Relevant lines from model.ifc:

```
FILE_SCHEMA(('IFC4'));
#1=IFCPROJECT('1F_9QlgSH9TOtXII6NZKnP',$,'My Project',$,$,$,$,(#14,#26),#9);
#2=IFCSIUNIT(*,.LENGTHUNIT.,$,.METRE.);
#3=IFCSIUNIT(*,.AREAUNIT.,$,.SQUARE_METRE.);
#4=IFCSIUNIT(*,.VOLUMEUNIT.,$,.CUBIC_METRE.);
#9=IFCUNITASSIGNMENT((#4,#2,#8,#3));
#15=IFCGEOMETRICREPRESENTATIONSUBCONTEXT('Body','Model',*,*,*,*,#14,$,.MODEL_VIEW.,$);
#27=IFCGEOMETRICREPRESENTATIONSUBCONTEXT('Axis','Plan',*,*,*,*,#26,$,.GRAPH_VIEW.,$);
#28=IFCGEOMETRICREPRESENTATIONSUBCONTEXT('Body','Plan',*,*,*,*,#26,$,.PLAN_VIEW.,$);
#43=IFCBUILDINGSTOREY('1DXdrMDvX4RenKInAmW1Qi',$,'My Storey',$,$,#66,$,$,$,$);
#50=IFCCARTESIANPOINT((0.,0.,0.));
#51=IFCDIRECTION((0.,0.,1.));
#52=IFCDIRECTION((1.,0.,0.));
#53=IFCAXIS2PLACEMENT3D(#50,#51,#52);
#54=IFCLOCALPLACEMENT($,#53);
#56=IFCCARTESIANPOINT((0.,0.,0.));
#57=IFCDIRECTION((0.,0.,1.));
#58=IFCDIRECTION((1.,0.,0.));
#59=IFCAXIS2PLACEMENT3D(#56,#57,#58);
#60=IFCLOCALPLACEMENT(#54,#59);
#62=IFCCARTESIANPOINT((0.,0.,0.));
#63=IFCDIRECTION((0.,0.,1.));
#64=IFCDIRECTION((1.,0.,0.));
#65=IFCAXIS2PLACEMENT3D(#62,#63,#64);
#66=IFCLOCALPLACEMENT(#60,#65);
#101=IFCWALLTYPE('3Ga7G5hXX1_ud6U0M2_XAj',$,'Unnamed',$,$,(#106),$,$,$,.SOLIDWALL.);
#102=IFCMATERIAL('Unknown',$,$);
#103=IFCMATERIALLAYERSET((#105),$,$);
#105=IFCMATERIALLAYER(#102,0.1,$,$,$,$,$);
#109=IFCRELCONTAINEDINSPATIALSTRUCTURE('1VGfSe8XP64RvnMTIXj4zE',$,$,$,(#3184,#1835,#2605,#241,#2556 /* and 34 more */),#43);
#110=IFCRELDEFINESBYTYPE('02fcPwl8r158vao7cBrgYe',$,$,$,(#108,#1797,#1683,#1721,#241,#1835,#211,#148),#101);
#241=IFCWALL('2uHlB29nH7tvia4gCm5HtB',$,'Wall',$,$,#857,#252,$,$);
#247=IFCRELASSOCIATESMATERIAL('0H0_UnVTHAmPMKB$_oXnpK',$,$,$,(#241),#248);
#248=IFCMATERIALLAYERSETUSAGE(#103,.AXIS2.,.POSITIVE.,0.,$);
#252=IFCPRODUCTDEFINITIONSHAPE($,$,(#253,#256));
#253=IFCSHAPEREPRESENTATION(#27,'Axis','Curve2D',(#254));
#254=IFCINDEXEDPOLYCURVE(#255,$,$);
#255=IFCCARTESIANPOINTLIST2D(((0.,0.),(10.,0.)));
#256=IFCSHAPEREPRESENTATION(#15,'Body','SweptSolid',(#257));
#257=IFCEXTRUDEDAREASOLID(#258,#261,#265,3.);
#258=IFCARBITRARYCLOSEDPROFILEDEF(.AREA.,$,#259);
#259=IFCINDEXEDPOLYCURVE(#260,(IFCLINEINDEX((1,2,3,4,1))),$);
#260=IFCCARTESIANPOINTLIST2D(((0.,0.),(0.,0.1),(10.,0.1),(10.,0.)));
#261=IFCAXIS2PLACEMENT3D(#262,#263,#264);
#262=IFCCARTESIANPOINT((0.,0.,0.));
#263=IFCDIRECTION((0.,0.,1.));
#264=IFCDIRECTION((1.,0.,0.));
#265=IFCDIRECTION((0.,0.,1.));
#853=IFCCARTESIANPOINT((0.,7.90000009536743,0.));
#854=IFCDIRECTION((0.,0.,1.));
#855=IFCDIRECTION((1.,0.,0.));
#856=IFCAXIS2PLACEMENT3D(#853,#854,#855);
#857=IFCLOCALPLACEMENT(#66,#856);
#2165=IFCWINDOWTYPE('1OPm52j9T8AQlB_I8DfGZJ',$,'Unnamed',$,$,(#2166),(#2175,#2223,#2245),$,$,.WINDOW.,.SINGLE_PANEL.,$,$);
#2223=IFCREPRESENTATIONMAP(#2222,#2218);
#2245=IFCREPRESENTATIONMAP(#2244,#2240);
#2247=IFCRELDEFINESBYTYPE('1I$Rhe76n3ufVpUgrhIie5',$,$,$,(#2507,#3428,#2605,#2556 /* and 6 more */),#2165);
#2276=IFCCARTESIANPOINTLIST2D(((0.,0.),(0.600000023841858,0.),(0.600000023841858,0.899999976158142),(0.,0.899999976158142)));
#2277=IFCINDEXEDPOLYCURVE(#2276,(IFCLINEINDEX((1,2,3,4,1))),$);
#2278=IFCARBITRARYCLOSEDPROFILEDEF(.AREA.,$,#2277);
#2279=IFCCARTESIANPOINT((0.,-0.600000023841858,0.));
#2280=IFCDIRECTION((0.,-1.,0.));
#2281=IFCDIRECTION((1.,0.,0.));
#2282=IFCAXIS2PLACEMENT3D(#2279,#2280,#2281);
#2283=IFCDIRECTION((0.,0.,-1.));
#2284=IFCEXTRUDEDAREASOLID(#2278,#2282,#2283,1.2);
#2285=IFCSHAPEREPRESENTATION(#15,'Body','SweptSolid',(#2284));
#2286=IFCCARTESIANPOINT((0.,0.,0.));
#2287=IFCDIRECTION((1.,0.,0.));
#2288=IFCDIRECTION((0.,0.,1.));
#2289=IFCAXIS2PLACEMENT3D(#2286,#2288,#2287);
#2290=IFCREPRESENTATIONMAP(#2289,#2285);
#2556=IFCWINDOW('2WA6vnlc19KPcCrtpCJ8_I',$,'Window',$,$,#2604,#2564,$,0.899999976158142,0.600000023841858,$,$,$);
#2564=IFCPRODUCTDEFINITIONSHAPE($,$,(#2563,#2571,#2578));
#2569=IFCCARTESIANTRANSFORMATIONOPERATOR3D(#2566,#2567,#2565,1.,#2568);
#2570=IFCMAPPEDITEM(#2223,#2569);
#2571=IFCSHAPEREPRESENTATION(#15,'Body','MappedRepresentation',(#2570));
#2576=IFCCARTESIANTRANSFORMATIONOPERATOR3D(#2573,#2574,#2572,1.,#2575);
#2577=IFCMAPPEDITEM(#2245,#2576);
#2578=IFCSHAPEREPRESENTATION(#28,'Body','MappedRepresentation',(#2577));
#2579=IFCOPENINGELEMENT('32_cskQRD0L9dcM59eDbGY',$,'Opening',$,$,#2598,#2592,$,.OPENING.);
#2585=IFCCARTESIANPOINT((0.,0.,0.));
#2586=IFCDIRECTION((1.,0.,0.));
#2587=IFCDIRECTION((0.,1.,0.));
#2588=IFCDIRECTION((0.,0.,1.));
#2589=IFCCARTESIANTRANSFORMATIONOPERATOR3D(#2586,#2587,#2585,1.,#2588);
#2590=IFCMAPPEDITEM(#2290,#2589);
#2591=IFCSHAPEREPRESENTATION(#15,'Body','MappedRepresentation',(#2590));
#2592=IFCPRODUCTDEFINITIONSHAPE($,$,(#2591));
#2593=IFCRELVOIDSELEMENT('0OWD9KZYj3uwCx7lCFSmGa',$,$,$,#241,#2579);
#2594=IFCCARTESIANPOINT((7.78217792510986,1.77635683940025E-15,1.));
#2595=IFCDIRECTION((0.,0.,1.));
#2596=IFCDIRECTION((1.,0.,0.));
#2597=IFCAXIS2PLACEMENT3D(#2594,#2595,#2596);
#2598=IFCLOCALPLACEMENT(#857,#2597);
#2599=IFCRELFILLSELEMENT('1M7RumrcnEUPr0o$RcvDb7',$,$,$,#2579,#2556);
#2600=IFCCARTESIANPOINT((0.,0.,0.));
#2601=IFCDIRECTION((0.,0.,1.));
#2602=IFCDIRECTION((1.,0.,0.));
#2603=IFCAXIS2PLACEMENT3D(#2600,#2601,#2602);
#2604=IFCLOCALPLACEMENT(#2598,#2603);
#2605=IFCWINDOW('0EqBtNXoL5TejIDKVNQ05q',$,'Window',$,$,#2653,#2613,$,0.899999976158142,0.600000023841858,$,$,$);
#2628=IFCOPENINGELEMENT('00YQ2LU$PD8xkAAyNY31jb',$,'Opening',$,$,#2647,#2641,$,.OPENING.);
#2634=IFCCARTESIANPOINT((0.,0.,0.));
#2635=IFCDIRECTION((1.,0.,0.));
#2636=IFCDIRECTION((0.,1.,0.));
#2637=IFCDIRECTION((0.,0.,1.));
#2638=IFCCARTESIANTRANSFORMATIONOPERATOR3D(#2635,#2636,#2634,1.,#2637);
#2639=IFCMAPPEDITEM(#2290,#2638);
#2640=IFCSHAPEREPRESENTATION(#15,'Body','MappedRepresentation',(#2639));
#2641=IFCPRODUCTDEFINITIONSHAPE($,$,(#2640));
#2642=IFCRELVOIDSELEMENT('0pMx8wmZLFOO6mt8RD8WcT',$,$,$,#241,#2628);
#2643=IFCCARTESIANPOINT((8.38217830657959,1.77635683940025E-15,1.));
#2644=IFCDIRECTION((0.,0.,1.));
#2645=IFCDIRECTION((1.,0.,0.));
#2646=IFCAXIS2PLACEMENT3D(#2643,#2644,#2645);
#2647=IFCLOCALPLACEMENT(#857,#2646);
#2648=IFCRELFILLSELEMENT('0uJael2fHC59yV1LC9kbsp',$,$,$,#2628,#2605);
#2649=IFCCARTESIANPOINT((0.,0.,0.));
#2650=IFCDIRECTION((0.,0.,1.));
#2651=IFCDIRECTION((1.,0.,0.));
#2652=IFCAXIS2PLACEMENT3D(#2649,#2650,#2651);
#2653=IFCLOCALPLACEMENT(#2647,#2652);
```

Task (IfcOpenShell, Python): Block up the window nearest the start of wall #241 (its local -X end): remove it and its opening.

```python
import ifcopenshell
import ifcopenshell.api.feature
import ifcopenshell.api.root
import ifcopenshell.geom
import ifcopenshell.util.shape

model = ifcopenshell.open("model.ifc")
settings = ifcopenshell.geom.settings()


def volume(element):
    """Net volume in cubic metres, openings subtracted."""
    shape = ifcopenshell.geom.create_shape(settings, element)
    return ifcopenshell.util.shape.get_volume(shape.geometry)


window = model.by_id(2556)
opening = window.FillsVoids[0].RelatingOpeningElement
wall = opening.VoidsElements[0].RelatingBuildingElement
before = volume(wall)

ifcopenshell.api.root.remove_product(model, product=window)
ifcopenshell.api.feature.remove_feature(model, feature=opening)

after = volume(wall)

print(f"wall volume {before:.3f} -> {after:.3f} m3")

model.write("model_rev.ifc")
```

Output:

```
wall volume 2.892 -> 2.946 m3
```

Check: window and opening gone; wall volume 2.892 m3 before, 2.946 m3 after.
